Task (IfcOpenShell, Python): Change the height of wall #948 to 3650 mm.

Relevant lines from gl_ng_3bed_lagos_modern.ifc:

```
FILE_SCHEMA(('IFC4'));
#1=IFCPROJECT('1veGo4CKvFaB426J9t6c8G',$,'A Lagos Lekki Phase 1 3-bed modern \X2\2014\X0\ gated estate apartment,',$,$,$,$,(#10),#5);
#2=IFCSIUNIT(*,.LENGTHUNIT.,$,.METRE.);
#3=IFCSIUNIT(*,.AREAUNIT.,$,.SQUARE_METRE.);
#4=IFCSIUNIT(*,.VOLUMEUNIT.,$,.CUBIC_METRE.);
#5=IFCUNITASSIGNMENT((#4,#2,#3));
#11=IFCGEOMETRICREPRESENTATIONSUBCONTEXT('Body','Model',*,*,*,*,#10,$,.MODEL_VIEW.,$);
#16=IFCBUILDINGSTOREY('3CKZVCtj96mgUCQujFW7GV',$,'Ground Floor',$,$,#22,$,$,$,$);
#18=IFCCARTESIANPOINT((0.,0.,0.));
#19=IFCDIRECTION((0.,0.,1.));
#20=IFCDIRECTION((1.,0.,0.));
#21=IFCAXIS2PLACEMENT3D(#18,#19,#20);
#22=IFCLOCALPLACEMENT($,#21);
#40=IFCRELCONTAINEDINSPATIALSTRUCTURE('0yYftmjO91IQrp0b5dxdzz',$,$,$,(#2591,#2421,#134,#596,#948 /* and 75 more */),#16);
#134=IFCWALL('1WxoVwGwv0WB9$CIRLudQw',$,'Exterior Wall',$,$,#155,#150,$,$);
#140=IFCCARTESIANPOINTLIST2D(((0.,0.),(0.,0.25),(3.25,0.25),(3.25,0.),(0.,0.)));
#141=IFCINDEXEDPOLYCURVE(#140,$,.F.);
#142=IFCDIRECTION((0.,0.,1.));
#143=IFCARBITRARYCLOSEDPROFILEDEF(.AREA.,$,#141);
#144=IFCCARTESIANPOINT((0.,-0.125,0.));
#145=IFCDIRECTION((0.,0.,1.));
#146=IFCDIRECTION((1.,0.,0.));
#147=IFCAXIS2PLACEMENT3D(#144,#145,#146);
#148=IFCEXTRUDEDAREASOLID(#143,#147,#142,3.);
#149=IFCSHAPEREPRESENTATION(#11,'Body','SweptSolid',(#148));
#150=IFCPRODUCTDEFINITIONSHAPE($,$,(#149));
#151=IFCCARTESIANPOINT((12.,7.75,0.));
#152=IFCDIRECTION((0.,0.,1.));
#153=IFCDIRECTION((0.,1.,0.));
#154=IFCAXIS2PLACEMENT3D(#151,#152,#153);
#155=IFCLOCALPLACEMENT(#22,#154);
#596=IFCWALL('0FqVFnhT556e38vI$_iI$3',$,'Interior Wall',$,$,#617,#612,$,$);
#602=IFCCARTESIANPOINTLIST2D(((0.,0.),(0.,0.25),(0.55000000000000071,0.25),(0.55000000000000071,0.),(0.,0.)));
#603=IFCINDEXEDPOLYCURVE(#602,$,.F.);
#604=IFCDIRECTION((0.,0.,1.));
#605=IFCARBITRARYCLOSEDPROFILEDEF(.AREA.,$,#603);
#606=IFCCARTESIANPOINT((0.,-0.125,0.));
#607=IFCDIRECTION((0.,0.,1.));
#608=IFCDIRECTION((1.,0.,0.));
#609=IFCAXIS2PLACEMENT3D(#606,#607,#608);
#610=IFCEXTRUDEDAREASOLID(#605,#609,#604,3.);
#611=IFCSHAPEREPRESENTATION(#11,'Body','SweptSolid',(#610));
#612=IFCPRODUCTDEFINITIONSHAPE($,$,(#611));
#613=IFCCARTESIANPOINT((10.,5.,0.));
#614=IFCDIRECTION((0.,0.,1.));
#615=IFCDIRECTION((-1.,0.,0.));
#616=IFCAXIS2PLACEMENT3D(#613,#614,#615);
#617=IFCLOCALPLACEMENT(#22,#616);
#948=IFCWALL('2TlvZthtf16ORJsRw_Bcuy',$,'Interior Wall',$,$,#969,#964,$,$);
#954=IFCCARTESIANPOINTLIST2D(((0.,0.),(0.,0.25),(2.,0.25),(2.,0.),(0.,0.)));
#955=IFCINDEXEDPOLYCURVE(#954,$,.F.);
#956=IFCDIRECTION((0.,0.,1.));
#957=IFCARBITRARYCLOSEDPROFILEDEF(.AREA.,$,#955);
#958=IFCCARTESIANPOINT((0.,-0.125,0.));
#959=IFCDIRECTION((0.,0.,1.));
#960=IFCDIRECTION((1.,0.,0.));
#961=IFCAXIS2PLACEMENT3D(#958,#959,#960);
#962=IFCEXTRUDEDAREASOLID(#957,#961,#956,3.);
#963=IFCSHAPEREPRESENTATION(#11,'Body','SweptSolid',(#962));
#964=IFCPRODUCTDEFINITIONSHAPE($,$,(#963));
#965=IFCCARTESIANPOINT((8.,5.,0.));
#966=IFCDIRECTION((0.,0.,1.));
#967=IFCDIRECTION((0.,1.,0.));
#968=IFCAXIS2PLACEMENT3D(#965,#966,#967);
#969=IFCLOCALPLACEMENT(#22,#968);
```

```python
import ifcopenshell
import ifcopenshell.geom
import ifcopenshell.util.representation
import ifcopenshell.util.shape
import ifcopenshell.util.unit

model = ifcopenshell.open("gl_ng_3bed_lagos_modern.ifc")
unit_scale = ifcopenshell.util.unit.calculate_unit_scale(model)
settings = ifcopenshell.geom.settings()


def volume(element):
    """Net volume in cubic metres, openings subtracted."""
    shape = ifcopenshell.geom.create_shape(settings, element)
    return ifcopenshell.util.shape.get_volume(shape.geometry)


wall = model.by_guid("2TlvZthtf16ORJsRw_Bcuy")
before = volume(wall)

body = ifcopenshell.util.representation.get_representation(wall, "Model", "Body")
solid = body.Items[0]
old_height = solid.Depth
solid.Depth = 3.65 / unit_scale
after = volume(wall)

print(f"height {old_height:g} -> {solid.Depth:g}, volume {before:.3f} -> {after:.3f} m3")

model.write("gl_ng_3bed_lagos_modern-out.ifc")
```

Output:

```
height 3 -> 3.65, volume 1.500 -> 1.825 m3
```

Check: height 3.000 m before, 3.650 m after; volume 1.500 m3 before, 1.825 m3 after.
